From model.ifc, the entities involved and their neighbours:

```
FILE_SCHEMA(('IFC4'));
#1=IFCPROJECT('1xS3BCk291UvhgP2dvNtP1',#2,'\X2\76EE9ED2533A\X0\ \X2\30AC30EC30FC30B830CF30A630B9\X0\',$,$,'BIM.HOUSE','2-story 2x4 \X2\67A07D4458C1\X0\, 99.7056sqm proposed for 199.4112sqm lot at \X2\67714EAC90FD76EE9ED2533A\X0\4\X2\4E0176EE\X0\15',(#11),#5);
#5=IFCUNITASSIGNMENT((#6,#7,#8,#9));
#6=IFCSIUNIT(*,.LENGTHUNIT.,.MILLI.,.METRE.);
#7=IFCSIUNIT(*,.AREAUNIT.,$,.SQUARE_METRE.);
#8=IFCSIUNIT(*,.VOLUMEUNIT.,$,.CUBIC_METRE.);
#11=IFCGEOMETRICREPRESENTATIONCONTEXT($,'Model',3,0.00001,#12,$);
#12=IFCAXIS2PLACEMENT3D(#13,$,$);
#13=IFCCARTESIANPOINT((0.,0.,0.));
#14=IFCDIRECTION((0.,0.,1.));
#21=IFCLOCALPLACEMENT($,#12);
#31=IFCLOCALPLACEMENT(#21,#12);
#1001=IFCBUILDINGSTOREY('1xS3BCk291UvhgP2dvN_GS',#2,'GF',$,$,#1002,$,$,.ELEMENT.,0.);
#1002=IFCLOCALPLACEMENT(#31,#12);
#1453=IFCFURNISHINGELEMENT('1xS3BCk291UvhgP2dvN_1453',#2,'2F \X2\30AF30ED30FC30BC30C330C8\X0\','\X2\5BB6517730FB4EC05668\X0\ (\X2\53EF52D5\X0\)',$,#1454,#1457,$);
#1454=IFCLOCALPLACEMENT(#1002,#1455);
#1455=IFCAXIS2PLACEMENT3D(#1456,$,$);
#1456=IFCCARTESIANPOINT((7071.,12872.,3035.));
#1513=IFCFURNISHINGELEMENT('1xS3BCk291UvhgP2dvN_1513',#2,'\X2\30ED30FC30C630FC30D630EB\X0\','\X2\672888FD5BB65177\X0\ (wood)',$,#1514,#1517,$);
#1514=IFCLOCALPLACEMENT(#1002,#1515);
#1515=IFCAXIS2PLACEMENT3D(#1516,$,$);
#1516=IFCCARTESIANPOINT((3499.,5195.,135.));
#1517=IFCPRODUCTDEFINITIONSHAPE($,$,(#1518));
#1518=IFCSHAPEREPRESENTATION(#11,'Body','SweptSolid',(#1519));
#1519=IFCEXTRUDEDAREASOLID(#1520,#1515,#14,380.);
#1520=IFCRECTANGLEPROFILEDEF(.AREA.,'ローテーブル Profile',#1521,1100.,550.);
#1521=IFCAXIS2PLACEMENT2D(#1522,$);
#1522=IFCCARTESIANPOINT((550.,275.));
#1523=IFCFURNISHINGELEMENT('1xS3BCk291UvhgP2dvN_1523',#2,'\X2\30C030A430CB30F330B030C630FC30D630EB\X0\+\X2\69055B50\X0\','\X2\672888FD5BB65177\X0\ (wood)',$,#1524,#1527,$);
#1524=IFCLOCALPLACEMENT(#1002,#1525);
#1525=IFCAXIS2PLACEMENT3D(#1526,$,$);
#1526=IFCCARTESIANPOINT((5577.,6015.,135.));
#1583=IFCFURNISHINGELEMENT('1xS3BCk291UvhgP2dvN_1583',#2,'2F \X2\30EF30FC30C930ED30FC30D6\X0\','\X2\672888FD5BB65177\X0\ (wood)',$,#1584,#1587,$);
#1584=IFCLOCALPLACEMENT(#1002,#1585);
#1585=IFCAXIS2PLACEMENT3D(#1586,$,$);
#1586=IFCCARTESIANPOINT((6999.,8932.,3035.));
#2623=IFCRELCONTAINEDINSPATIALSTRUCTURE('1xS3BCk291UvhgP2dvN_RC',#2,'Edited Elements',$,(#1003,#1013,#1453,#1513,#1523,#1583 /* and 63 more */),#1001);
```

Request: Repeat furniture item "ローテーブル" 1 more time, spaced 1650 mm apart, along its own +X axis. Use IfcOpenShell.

```python
import ifcopenshell
import ifcopenshell.api.geometry
import ifcopenshell.api.root
import ifcopenshell.util.element
import ifcopenshell.util.placement
import ifcopenshell.util.unit

model = ifcopenshell.open("model.ifc")
unit_scale = ifcopenshell.util.unit.calculate_unit_scale(model)


def reuse_history(source, copy):
    """copy_class also copies each property set's owner history, people and application; keep the originals."""
    for rel in copy.IsDefinedBy:
        if rel.is_a("IfcRelDefinesByProperties") and (history := rel.RelatingPropertyDefinition.OwnerHistory):
            rel.RelatingPropertyDefinition.OwnerHistory = source.OwnerHistory
            ifcopenshell.util.element.remove_deep2(model, history)


source = model.by_guid("1xS3BCk291UvhgP2dvN_1513")
base = ifcopenshell.util.placement.get_local_placement(source.ObjectPlacement)
step = base[:3, 0] * 1.65 / unit_scale

for i in range(1, 2):
    copy = ifcopenshell.api.root.copy_class(model, product=source)
    copy.Representation = ifcopenshell.util.element.copy_deep(
        model, source.Representation, exclude=["IfcGeometricRepresentationContext", "IfcRepresentationMap"]
    )
    reuse_history(source, copy)
    matrix = base.copy()
    matrix[:3, 3] += i * step
    print("added at", matrix[:3, 3].round(3) + 0.0)
    ifcopenshell.api.geometry.edit_object_placement(model, product=copy, matrix=matrix, is_si=False)

model.write("model_updated.ifc")
```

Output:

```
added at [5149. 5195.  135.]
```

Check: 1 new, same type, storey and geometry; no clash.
